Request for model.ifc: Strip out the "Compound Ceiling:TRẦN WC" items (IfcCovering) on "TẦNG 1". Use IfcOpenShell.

First a look at what the model holds.

```python
import ifcopenshell
import ifcopenshell.util.element

model = ifcopenshell.open("model.ifc")
print(model.schema)
storey = next(s for s in model.by_type("IfcBuildingStorey") if s.Name == "TẦNG 1")
coverings = [e for e in ifcopenshell.util.element.get_decomposition(storey) if e.is_a("IfcCovering")]
seen = {}
for e in coverings:
    element_type = ifcopenshell.util.element.get_type(e)
    name = element_type.Name if element_type not in (None, e) else None
    seen[name] = seen.get(name, 0) + 1
for name, count in sorted(seen.items(), key=str):
    print(count, "x", name)
```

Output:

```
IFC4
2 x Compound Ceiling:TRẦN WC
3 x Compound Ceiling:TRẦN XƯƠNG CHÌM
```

```python
import ifcopenshell
import ifcopenshell.api.root
import ifcopenshell.util.element

model = ifcopenshell.open("model.ifc")

storey = next(s for s in model.by_type("IfcBuildingStorey") if s.Name == "TẦNG 1")
coverings = [e for e in ifcopenshell.util.element.get_decomposition(storey) if e.is_a("IfcCovering")]
targets = [e for e in coverings if (t := ifcopenshell.util.element.get_type(e)) not in (None, e) and t.Name == "Compound Ceiling:TRẦN WC"]

for e in targets:
    ifcopenshell.api.root.remove_product(model, product=e)
print(len(targets), "removed")

model.write("model-out.ifc")
```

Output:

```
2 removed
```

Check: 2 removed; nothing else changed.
